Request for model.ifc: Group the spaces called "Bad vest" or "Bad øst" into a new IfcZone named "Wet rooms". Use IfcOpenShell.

First a look at what the model holds.

```python
import ifcopenshell

model = ifcopenshell.open("model.ifc")
print(model.schema)
seen = {}
for space in model.by_type("IfcSpace"):
    seen[space.LongName] = seen.get(space.LongName, 0) + 1
for name, count in sorted(seen.items(), key=str):
    print(count, "x", name)
print("zones:", [z.Name for z in model.by_type("IfcZone")][:20])
```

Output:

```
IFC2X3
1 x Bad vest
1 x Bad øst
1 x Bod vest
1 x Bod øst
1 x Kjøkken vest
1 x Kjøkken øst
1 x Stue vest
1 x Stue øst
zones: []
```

```python
import ifcopenshell
import ifcopenshell.api.group
import ifcopenshell.api.root

model = ifcopenshell.open("model.ifc")

names = {"Bad vest", "Bad øst"}
spaces = [s for s in model.by_type("IfcSpace") if s.LongName in names]

zone = ifcopenshell.api.root.create_entity(model, ifc_class="IfcZone", name="Wet rooms")
ifcopenshell.api.group.assign_group(model, products=spaces, group=zone)
print(len(spaces), "spaces in", zone.Name)

model.write("model-out.ifc")
```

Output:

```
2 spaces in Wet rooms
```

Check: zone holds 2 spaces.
